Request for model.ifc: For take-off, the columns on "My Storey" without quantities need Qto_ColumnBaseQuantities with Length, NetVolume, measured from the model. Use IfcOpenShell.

First a look at what the model holds.

```python
import ifcopenshell
import ifcopenshell.util.element
import ifcopenshell.util.unit

model = ifcopenshell.open("model.ifc")
print(model.schema)
for unit_type in ("LENGTHUNIT", "AREAUNIT", "VOLUMEUNIT"):
    print(unit_type, ifcopenshell.util.unit.calculate_unit_scale(model, unit_type))
storey = next(s for s in model.by_type("IfcBuildingStorey") if s.Name == "My Storey")
columns = [e for e in ifcopenshell.util.element.get_decomposition(storey) if e.is_a("IfcColumn")]
for e in sorted(columns, key=lambda e: e.id()):
    print(e.id(), e.is_a(), e.Name, list(ifcopenshell.util.element.get_psets(e, qtos_only=True)), sep=" | ")
```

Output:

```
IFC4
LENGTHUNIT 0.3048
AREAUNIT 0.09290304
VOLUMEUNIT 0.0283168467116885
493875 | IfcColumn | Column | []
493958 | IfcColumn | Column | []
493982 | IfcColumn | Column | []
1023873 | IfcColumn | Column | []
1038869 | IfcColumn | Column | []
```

```python
import ifcopenshell
import ifcopenshell.api.pset
import ifcopenshell.geom
import ifcopenshell.util.element
import ifcopenshell.util.shape
import ifcopenshell.util.unit

model = ifcopenshell.open("model.ifc")
unit_scale = ifcopenshell.util.unit.calculate_unit_scale(model)
volume_scale = ifcopenshell.util.unit.calculate_unit_scale(model, "VOLUMEUNIT")
settings = ifcopenshell.geom.settings()

storey = next(s for s in model.by_type("IfcBuildingStorey") if s.Name == "My Storey")
columns = [e for e in ifcopenshell.util.element.get_decomposition(storey) if e.is_a("IfcColumn")]

for e in sorted(columns, key=lambda e: e.id()):
    if ifcopenshell.util.element.get_psets(e, qtos_only=True, should_inherit=False):
        continue
    # Geometry comes back in metres, in the element's own axes.
    shape = ifcopenshell.geom.create_shape(settings, e)
    values = {
        "Length": ifcopenshell.util.shape.get_z(shape.geometry) / unit_scale,
        "NetVolume": ifcopenshell.util.shape.get_volume(shape.geometry) / volume_scale,
    }
    qto = ifcopenshell.api.pset.add_qto(model, product=e, name="Qto_ColumnBaseQuantities")
    ifcopenshell.api.pset.edit_qto(model, qto=qto, properties=values)
    print(e.id(), {k: round(v, 3) for k, v in values.items()})

model.write("model_updated.ifc")
```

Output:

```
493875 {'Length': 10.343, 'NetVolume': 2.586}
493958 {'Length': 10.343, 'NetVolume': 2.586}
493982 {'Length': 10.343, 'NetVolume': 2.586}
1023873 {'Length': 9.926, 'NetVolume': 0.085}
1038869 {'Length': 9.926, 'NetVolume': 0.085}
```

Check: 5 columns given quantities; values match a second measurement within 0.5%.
